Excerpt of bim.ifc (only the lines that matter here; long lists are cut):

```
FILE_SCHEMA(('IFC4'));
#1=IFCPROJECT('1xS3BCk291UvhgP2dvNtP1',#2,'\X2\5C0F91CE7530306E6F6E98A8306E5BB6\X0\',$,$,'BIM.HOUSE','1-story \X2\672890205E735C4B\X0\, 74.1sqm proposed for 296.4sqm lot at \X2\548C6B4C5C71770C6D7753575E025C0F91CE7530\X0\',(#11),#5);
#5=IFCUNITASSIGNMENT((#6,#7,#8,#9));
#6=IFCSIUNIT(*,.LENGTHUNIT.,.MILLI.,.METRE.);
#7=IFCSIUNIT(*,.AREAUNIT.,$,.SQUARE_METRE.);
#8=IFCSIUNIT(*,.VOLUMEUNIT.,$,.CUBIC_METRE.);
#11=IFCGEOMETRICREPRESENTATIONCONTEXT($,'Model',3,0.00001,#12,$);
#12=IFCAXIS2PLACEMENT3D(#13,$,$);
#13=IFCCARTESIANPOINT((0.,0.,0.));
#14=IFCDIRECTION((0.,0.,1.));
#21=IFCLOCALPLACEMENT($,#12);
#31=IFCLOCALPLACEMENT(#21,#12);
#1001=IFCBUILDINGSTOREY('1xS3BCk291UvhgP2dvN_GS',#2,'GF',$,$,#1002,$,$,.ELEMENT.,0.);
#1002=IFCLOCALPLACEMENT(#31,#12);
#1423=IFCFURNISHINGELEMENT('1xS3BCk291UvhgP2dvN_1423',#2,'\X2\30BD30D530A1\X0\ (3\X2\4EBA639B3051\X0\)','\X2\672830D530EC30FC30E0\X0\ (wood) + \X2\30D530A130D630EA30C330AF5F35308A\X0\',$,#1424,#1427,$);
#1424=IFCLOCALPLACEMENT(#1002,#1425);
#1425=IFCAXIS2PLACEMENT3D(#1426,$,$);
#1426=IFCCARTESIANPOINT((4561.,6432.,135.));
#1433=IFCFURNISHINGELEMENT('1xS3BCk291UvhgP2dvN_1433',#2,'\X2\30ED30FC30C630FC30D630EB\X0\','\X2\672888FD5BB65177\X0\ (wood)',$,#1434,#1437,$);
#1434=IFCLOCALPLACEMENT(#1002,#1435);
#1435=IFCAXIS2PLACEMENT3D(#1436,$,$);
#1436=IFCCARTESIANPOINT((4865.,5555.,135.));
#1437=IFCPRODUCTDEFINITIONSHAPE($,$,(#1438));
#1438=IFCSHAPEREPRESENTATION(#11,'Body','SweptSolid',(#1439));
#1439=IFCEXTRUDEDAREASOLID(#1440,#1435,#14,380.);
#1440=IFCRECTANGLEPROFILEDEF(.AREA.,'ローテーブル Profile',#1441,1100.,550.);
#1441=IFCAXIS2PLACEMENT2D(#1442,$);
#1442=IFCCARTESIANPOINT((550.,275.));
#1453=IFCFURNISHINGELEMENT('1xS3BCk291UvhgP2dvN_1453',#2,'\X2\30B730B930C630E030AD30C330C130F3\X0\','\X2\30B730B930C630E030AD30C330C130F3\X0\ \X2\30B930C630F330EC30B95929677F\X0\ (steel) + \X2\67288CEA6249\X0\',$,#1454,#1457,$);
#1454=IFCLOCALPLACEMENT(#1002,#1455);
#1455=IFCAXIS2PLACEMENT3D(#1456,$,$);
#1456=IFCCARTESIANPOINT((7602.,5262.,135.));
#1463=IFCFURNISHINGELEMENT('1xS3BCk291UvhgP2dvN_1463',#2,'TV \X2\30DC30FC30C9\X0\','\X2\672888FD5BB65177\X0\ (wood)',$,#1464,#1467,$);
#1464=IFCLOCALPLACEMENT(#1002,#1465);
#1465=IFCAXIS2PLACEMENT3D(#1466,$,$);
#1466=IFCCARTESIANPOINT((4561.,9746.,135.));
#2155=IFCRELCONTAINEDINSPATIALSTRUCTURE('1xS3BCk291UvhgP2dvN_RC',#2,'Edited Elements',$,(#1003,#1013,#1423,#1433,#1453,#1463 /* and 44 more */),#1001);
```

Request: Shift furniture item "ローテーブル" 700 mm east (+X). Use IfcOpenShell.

```python
import ifcopenshell
import ifcopenshell.api.geometry
import ifcopenshell.util.placement

model = ifcopenshell.open("bim.ifc")

item = model.by_guid("1xS3BCk291UvhgP2dvN_1433")
matrix = ifcopenshell.util.placement.get_local_placement(item.ObjectPlacement)
matrix[0, 3] += 700.0
ifcopenshell.api.geometry.edit_object_placement(model, product=item, matrix=matrix, is_si=False)

print(ifcopenshell.util.placement.get_local_placement(item.ObjectPlacement).round(3) + 0.0)

model.write("bim_edited.ifc")
```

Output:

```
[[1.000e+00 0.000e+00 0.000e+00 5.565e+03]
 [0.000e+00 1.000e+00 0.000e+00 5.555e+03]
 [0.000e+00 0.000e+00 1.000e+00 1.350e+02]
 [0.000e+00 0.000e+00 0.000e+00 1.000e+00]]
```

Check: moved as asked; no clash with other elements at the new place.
